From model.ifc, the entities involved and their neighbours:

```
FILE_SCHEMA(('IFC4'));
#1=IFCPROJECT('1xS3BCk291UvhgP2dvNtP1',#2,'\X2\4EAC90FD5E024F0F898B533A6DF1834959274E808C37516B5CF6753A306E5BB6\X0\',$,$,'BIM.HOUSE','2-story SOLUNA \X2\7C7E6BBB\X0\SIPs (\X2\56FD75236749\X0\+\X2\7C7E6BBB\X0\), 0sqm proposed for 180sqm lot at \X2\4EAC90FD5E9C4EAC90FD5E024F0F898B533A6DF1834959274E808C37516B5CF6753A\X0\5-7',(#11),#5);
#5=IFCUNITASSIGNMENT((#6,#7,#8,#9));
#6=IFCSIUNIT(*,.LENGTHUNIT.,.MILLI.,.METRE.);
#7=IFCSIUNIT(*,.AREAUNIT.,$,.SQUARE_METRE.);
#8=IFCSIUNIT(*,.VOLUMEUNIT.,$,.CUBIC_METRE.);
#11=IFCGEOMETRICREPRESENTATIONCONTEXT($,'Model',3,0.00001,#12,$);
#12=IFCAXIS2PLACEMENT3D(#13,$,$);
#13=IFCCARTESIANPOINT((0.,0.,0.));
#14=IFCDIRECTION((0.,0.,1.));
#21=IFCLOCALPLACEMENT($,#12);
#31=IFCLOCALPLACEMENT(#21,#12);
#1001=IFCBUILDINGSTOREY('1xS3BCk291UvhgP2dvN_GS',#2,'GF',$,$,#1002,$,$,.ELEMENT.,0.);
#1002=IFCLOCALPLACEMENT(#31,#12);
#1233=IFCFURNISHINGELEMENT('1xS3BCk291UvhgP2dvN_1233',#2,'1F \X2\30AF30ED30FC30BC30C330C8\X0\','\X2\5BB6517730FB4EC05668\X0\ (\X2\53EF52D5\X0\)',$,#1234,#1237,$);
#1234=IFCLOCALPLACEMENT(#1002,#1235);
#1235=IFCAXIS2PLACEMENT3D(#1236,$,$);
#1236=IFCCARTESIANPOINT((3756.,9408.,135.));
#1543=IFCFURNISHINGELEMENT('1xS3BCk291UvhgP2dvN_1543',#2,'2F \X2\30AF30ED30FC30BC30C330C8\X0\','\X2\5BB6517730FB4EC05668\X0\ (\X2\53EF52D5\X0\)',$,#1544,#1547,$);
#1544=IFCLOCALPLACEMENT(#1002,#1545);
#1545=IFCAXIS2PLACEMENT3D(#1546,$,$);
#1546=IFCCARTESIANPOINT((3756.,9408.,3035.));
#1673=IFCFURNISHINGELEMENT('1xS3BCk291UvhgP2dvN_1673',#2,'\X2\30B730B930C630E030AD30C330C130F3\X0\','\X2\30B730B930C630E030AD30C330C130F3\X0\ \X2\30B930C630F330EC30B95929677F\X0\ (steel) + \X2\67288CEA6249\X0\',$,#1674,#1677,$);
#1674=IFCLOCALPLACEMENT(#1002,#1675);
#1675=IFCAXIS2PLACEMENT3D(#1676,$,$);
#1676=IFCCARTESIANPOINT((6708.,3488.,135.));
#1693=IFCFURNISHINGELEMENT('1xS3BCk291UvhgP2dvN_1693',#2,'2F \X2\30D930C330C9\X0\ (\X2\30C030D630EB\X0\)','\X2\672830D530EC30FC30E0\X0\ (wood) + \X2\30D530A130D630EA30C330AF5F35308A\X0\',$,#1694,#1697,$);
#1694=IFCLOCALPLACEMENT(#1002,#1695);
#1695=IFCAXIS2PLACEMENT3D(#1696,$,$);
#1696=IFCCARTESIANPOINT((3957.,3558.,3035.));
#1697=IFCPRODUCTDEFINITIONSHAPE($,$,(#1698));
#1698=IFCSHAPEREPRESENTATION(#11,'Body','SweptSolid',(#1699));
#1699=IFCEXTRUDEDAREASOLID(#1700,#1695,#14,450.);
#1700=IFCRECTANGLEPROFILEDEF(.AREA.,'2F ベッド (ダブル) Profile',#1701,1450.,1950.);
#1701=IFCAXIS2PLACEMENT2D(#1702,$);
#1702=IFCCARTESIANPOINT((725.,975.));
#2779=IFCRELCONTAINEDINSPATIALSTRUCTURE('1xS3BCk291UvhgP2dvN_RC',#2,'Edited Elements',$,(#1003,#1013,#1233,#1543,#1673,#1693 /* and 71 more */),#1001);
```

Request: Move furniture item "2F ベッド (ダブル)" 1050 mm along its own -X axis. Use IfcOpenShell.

```python
import ifcopenshell
import ifcopenshell.api.geometry
import ifcopenshell.util.placement
import ifcopenshell.util.unit

model = ifcopenshell.open("model.ifc")
unit_scale = ifcopenshell.util.unit.calculate_unit_scale(model)

item = model.by_id(1693)
matrix = ifcopenshell.util.placement.get_local_placement(item.ObjectPlacement)
matrix[:3, 3] -= matrix[:3, 0] * 1.05 / unit_scale
ifcopenshell.api.geometry.edit_object_placement(model, product=item, matrix=matrix, is_si=False)

print(ifcopenshell.util.placement.get_local_placement(item.ObjectPlacement).round(3) + 0.0)

model.write("model_updated.ifc")
```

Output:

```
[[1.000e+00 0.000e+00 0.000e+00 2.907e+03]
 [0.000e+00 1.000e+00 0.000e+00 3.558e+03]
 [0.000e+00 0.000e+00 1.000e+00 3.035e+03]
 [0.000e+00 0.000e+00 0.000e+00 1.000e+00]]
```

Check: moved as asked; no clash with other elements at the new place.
